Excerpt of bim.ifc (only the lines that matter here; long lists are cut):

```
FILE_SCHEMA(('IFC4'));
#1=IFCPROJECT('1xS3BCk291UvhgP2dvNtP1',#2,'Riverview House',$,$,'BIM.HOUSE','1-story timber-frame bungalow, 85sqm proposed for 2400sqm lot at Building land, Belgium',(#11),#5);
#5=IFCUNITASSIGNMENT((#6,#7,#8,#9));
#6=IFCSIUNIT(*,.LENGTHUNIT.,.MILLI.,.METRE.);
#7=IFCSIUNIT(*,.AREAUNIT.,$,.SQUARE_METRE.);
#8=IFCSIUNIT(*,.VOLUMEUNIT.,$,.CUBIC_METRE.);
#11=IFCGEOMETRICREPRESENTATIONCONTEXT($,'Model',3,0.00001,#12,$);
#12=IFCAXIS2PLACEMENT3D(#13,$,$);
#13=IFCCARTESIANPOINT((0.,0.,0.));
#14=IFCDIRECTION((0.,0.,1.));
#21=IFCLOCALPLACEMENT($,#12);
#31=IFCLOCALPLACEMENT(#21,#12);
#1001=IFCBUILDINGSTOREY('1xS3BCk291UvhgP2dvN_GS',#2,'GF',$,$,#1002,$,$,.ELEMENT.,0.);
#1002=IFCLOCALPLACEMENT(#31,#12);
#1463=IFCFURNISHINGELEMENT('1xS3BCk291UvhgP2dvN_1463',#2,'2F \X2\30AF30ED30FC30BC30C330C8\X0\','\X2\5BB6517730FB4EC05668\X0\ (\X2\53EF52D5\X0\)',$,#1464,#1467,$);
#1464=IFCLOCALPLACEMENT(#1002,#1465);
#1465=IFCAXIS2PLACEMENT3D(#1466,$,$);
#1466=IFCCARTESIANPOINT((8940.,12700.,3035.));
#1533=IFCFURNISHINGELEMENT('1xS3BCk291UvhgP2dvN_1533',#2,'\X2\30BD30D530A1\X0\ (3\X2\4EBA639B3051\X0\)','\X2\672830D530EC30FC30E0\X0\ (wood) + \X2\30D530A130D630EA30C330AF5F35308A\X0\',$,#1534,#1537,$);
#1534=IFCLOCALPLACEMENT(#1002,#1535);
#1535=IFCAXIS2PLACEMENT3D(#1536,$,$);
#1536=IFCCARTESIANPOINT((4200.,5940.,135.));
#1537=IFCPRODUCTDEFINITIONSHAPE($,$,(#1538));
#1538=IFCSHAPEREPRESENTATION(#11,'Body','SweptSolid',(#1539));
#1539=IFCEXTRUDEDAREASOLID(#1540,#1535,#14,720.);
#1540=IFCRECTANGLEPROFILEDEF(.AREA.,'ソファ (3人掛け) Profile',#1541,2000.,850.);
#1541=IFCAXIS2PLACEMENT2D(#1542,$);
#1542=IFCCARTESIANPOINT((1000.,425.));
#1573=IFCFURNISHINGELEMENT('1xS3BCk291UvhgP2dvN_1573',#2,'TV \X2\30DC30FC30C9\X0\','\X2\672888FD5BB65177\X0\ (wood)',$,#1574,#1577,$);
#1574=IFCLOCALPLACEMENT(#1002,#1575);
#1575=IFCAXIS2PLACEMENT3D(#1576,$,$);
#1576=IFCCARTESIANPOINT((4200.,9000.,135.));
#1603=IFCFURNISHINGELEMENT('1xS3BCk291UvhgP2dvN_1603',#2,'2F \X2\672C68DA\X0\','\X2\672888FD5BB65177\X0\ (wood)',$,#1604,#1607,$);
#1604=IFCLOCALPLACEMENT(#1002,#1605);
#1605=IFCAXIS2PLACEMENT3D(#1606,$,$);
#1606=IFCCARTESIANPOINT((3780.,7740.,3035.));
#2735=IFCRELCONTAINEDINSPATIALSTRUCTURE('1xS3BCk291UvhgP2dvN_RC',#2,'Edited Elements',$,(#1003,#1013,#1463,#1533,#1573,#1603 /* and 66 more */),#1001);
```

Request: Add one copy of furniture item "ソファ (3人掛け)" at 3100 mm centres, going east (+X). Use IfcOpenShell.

```python
import numpy as np
import ifcopenshell
import ifcopenshell.api.geometry
import ifcopenshell.api.root
import ifcopenshell.util.element
import ifcopenshell.util.placement

model = ifcopenshell.open("bim.ifc")


def reuse_history(source, copy):
    """copy_class also copies each property set's owner history, people and application; keep the originals."""
    for rel in copy.IsDefinedBy:
        if rel.is_a("IfcRelDefinesByProperties") and (history := rel.RelatingPropertyDefinition.OwnerHistory):
            rel.RelatingPropertyDefinition.OwnerHistory = source.OwnerHistory
            ifcopenshell.util.element.remove_deep2(model, history)


source = model.by_id(1533)
base = ifcopenshell.util.placement.get_local_placement(source.ObjectPlacement)
step = np.array([1.0, 0.0, 0.0]) * 3100.0

for i in range(1, 2):
    copy = ifcopenshell.api.root.copy_class(model, product=source)
    copy.Representation = ifcopenshell.util.element.copy_deep(
        model, source.Representation, exclude=["IfcGeometricRepresentationContext", "IfcRepresentationMap"]
    )
    reuse_history(source, copy)
    matrix = base.copy()
    matrix[:3, 3] += i * step
    print("added at", matrix[:3, 3].round(3) + 0.0)
    ifcopenshell.api.geometry.edit_object_placement(model, product=copy, matrix=matrix, is_si=False)

model.write("bim_v2.ifc")
```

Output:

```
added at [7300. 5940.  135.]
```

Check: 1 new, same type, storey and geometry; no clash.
